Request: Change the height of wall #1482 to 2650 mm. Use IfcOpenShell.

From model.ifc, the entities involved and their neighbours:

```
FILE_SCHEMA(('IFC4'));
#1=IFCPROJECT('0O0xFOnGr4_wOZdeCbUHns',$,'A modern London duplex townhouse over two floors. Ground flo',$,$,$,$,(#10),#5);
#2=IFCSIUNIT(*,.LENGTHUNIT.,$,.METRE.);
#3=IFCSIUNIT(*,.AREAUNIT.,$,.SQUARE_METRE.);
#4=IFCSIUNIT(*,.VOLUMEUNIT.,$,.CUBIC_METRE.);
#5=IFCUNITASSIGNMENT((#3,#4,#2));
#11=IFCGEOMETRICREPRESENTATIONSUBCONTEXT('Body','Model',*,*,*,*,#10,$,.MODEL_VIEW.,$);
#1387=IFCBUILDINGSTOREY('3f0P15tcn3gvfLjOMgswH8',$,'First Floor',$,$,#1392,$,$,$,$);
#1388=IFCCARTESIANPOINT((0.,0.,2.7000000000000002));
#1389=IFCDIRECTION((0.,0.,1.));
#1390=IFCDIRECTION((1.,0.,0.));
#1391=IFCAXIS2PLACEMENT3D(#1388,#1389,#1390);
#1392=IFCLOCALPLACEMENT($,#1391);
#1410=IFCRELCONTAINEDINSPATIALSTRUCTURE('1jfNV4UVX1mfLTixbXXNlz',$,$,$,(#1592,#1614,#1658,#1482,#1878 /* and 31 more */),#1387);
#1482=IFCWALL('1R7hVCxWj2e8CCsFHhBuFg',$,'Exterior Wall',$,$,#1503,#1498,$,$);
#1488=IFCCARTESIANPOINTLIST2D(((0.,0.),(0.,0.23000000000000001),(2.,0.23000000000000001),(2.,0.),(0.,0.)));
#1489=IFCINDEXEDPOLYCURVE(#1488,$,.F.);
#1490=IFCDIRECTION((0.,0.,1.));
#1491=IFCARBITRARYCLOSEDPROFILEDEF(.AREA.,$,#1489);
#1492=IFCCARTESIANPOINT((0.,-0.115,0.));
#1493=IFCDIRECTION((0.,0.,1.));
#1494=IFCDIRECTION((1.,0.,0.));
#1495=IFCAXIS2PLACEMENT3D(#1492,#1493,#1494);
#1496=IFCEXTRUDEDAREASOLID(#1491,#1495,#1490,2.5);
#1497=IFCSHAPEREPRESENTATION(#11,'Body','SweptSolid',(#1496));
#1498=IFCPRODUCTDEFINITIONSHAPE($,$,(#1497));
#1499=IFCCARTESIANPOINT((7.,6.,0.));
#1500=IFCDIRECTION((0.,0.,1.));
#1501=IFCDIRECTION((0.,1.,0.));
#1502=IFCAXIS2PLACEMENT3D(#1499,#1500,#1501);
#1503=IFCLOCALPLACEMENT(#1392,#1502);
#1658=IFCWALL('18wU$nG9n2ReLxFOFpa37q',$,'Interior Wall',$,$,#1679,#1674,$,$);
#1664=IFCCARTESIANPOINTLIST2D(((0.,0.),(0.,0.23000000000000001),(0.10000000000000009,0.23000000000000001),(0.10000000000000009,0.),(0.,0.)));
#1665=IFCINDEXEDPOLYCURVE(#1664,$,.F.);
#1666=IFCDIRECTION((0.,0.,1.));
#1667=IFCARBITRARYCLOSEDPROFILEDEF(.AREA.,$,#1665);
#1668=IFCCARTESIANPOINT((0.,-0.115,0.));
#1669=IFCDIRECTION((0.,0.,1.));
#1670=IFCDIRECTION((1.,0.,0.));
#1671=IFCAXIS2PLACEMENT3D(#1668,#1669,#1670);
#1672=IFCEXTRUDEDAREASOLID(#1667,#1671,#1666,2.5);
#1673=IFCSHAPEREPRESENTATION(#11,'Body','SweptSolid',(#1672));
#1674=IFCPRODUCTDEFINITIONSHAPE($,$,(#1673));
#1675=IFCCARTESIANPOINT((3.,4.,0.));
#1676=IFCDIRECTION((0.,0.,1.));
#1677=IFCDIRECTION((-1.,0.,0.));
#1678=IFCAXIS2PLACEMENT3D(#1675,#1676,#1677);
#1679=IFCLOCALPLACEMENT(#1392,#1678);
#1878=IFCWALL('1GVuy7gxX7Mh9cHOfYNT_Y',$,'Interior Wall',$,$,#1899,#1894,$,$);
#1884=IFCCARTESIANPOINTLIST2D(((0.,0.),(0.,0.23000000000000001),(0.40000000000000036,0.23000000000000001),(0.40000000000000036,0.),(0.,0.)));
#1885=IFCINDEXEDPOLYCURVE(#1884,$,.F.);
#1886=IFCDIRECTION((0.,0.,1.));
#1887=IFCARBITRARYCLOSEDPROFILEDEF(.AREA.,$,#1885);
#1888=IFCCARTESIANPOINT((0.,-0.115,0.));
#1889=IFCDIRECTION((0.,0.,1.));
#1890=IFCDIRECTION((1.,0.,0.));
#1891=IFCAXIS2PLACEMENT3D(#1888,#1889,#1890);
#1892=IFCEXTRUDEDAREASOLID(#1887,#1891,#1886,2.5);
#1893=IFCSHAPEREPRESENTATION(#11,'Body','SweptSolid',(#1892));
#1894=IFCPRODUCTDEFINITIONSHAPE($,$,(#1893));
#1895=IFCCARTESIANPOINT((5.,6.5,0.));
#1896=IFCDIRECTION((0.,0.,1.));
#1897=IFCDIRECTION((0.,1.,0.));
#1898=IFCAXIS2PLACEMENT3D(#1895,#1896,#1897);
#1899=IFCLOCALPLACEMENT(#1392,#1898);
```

```python
import ifcopenshell
import ifcopenshell.geom
import ifcopenshell.util.representation
import ifcopenshell.util.shape
import ifcopenshell.util.unit

model = ifcopenshell.open("model.ifc")
unit_scale = ifcopenshell.util.unit.calculate_unit_scale(model)
settings = ifcopenshell.geom.settings()


def volume(element):
    """Net volume in cubic metres, openings subtracted."""
    shape = ifcopenshell.geom.create_shape(settings, element)
    return ifcopenshell.util.shape.get_volume(shape.geometry)


wall = model.by_id(1482)
before = volume(wall)

body = ifcopenshell.util.representation.get_representation(wall, "Model", "Body")
solid = body.Items[0]
old_height = solid.Depth
solid.Depth = 2.65 / unit_scale
after = volume(wall)

print(f"height {old_height:g} -> {solid.Depth:g}, volume {before:.3f} -> {after:.3f} m3")

model.write("model_updated.ifc")
```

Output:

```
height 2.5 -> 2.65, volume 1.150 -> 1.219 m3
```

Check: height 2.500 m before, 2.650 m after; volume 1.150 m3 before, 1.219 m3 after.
